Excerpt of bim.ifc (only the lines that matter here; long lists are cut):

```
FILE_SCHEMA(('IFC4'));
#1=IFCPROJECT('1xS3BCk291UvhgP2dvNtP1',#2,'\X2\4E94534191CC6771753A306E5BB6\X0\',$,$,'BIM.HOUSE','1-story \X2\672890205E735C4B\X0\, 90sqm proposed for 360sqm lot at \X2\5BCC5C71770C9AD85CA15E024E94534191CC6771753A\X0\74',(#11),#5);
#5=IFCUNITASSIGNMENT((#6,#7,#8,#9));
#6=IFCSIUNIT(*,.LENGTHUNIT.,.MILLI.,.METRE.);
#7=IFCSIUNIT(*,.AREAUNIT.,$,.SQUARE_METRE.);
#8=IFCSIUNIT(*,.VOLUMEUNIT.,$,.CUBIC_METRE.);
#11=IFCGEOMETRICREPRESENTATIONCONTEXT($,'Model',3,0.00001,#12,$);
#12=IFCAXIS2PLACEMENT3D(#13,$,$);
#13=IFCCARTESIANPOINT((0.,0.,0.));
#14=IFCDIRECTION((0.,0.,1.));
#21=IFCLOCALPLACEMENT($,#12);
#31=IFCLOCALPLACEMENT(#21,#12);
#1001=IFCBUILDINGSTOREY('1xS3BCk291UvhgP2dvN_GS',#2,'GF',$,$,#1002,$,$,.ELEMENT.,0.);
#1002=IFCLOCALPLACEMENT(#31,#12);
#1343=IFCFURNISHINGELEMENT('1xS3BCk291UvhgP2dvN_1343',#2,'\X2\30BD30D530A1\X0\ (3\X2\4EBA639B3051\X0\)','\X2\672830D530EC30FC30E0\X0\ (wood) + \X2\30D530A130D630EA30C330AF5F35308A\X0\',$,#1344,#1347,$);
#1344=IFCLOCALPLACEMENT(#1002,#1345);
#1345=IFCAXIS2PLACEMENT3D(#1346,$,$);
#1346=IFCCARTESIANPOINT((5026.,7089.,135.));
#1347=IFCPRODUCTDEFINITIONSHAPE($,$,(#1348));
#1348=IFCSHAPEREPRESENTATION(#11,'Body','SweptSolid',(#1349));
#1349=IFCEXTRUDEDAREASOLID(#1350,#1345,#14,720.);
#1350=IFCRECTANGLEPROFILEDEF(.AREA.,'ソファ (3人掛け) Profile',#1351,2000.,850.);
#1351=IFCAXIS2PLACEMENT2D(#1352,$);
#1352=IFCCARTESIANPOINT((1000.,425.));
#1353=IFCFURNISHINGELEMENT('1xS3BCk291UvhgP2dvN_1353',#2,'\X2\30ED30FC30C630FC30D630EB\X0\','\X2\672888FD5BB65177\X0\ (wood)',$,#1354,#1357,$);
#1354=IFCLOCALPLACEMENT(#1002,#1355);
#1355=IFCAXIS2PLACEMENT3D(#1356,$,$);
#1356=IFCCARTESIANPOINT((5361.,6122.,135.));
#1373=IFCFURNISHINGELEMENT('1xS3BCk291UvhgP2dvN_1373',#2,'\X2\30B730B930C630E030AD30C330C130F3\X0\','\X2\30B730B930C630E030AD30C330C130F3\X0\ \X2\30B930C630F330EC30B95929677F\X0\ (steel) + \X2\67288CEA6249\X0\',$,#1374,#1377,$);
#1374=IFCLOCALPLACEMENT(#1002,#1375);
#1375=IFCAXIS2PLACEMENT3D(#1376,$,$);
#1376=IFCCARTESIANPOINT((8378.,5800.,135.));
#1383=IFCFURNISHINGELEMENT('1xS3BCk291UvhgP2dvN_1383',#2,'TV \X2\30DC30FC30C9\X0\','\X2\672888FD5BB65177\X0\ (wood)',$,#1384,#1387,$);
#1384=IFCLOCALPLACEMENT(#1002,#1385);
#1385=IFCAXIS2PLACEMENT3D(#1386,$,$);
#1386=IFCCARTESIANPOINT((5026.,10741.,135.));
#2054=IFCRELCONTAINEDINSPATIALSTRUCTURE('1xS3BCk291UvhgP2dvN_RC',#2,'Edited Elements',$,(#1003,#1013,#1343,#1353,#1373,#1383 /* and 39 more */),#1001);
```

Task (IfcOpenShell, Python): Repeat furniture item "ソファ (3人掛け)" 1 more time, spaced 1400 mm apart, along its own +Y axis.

```python
import ifcopenshell
import ifcopenshell.api.geometry
import ifcopenshell.api.root
import ifcopenshell.util.element
import ifcopenshell.util.placement
import ifcopenshell.util.unit

model = ifcopenshell.open("bim.ifc")
unit_scale = ifcopenshell.util.unit.calculate_unit_scale(model)


def reuse_history(source, copy):
    """copy_class also copies each property set's owner history, people and application; keep the originals."""
    for rel in copy.IsDefinedBy:
        if rel.is_a("IfcRelDefinesByProperties") and (history := rel.RelatingPropertyDefinition.OwnerHistory):
            rel.RelatingPropertyDefinition.OwnerHistory = source.OwnerHistory
            ifcopenshell.util.element.remove_deep2(model, history)


source = model.by_guid("1xS3BCk291UvhgP2dvN_1343")
base = ifcopenshell.util.placement.get_local_placement(source.ObjectPlacement)
step = base[:3, 1] * 1.4 / unit_scale

for i in range(1, 2):
    copy = ifcopenshell.api.root.copy_class(model, product=source)
    copy.Representation = ifcopenshell.util.element.copy_deep(
        model, source.Representation, exclude=["IfcGeometricRepresentationContext", "IfcRepresentationMap"]
    )
    reuse_history(source, copy)
    matrix = base.copy()
    matrix[:3, 3] += i * step
    print("added at", matrix[:3, 3].round(3) + 0.0)
    ifcopenshell.api.geometry.edit_object_placement(model, product=copy, matrix=matrix, is_si=False)

model.write("bim_updated.ifc")
```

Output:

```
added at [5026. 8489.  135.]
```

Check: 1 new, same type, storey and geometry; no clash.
